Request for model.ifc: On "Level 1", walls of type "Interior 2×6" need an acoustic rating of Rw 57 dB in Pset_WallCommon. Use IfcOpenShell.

First a look at what the model holds.

```python
import ifcopenshell
import ifcopenshell.util.element

model = ifcopenshell.open("model.ifc")
print(model.schema)
storey = next(s for s in model.by_type("IfcBuildingStorey") if s.Name == "Level 1")
walls = [e for e in ifcopenshell.util.element.get_decomposition(storey) if e.is_a("IfcWall")]
seen = {}
for e in walls:
    element_type = ifcopenshell.util.element.get_type(e)
    key = (element_type.Name if element_type != e and element_type else None, ifcopenshell.util.element.get_pset(e, "Pset_WallCommon", "AcousticRating"))
    seen[key] = seen.get(key, 0) + 1
for (name, value), count in sorted(seen.items(), key=str):
    print(count, "x", name, "|", value)
```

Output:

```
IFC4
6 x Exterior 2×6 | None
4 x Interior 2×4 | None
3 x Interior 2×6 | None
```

```python
import ifcopenshell
import ifcopenshell.api.pset
import ifcopenshell.util.element

model = ifcopenshell.open("model.ifc")

storey = next(s for s in model.by_type("IfcBuildingStorey") if s.Name == "Level 1")
walls = [e for e in ifcopenshell.util.element.get_decomposition(storey) if e.is_a("IfcWall")]

count = 0
for e in walls:
    element_type = ifcopenshell.util.element.get_type(e)
    if element_type in (None, e) or element_type.Name != "Interior 2×6":
        continue
    # add_pset returns the element's existing set when there is one.
    pset = ifcopenshell.api.pset.add_pset(model, product=e, name="Pset_WallCommon")
    ifcopenshell.api.pset.edit_pset(model, pset=pset, properties={"AcousticRating": "Rw 57 dB"})
    count += 1

print(count, "walls updated")

model.write("model_rev.ifc")
```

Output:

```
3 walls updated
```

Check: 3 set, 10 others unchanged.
